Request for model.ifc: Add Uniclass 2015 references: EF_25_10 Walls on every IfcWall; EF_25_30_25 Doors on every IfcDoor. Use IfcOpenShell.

First a look at what the model holds.

```python
import ifcopenshell

model = ifcopenshell.open("model.ifc")
print(model.schema)
print("classifications:", [c.Name for c in model.by_type("IfcClassification")])
for ifc_class in ("IfcDoor", "IfcRoof", "IfcStair", "IfcWall", "IfcWindow"):
    print(ifc_class, len(model.by_type(ifc_class)))
```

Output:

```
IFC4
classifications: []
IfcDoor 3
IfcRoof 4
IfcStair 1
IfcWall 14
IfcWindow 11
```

```python
import ifcopenshell
import ifcopenshell.api.classification

model = ifcopenshell.open("model.ifc")

system = ifcopenshell.api.classification.add_classification(model, classification="Uniclass 2015")

codes = {
    "IfcWall": ("EF_25_10", "Walls"),
    "IfcDoor": ("EF_25_30_25", "Doors"),
}
for ifc_class, (code, name) in codes.items():
    products = model.by_type(ifc_class)
    ifcopenshell.api.classification.add_reference(
        model, products=products, classification=system, identification=code, name=name
    )
    print(code, len(products))

model.write("model_rev.ifc")
```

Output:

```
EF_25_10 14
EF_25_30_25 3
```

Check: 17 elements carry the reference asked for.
